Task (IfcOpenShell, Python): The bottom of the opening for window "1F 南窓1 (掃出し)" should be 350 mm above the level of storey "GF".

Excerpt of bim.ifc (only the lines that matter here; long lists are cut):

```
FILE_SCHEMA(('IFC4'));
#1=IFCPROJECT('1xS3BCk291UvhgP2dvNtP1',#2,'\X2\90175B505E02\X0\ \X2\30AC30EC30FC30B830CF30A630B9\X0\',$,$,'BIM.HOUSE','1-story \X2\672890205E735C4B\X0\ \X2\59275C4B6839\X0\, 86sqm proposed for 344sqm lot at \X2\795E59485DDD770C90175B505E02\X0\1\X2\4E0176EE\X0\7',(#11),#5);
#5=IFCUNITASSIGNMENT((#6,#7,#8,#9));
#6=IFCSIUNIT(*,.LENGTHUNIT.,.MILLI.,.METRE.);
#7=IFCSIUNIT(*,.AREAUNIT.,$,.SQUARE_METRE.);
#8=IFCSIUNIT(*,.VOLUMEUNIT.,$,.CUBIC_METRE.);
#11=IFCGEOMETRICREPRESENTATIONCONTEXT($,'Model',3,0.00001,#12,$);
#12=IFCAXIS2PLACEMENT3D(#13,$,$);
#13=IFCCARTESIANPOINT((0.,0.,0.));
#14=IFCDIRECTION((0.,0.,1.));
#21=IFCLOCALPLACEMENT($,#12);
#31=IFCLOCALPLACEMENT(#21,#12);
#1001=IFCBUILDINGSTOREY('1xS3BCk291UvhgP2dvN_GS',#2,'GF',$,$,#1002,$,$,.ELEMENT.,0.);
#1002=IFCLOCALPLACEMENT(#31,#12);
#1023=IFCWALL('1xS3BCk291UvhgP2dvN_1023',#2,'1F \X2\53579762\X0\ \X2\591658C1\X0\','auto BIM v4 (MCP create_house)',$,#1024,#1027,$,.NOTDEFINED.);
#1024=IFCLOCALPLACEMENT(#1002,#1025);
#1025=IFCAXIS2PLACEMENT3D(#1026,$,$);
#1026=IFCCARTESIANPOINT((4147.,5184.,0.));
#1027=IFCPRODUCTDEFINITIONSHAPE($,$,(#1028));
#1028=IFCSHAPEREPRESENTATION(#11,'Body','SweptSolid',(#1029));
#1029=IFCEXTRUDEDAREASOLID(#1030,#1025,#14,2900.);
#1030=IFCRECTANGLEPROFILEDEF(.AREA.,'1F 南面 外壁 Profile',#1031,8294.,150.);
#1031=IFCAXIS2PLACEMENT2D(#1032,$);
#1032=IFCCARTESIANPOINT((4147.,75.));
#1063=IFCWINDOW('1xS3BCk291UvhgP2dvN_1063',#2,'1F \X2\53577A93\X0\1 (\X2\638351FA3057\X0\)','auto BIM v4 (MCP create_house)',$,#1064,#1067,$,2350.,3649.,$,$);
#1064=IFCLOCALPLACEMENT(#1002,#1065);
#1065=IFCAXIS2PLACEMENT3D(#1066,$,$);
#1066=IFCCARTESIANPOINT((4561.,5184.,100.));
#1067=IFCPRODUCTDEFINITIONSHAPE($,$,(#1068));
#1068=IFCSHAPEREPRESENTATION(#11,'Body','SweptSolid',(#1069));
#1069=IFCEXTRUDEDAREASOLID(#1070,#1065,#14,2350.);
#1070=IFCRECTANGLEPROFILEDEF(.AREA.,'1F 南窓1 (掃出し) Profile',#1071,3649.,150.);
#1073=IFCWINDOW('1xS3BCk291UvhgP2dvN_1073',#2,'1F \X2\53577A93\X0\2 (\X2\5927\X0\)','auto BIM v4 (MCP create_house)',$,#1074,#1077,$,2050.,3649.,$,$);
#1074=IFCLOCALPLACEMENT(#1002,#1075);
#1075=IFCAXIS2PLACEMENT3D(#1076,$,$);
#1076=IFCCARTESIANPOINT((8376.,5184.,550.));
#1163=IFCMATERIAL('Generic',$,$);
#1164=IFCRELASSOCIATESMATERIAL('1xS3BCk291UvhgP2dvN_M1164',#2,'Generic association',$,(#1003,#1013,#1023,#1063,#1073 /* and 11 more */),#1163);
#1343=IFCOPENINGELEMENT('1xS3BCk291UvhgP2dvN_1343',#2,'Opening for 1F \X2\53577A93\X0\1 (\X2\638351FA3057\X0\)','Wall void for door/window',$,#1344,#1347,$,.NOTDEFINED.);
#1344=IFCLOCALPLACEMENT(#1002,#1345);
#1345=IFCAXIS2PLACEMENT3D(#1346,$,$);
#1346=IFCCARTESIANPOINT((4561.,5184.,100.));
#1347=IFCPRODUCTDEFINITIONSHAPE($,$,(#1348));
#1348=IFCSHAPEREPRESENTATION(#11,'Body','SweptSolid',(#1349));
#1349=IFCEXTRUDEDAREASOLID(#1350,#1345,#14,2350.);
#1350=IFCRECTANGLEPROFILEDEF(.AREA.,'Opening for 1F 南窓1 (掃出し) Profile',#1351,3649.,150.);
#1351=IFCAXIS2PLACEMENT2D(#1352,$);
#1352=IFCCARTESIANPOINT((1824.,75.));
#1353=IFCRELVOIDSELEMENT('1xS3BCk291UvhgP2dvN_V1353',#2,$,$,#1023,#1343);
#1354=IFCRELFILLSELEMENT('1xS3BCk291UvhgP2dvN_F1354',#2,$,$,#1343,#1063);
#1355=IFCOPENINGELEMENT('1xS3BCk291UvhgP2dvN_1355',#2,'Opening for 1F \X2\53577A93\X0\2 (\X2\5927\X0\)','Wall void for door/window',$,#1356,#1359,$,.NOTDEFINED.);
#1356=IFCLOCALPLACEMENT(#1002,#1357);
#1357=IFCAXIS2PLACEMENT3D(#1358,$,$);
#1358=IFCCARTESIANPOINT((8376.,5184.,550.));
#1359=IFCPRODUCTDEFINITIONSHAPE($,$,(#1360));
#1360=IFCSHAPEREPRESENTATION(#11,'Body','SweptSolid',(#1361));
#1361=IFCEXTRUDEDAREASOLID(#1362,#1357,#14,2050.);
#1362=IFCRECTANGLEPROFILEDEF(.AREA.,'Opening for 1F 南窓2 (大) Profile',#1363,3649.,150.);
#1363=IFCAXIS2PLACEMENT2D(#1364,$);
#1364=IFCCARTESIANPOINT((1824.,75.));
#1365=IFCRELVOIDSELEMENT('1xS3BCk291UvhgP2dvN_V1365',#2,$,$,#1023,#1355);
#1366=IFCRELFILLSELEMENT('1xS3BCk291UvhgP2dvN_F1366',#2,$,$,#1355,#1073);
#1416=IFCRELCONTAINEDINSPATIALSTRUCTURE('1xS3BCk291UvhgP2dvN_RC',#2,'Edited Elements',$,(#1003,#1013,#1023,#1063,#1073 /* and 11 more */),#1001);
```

```python
import numpy as np
import ifcopenshell
import ifcopenshell.api.geometry
import ifcopenshell.geom
import ifcopenshell.util.element
import ifcopenshell.util.placement
import ifcopenshell.util.shape
import ifcopenshell.util.unit

model = ifcopenshell.open("bim.ifc")
unit_scale = ifcopenshell.util.unit.calculate_unit_scale(model)

window = model.by_guid("1xS3BCk291UvhgP2dvN_1063")
opening = window.FillsVoids[0].RelatingOpeningElement
storey = ifcopenshell.util.element.get_container(window, ifc_class="IfcBuildingStorey")
level = ifcopenshell.util.placement.get_local_placement(storey.ObjectPlacement)[2, 3]

# The opening's origin need not be at the sill, so measure its lowest point.
shape = ifcopenshell.geom.create_shape(ifcopenshell.geom.settings(), opening)
bottom = ifcopenshell.util.shape.get_shape_bottom_elevation(shape, shape.geometry) / unit_scale
dz = level + 350.0 - bottom

shift = np.array([0.0, 0.0, dz])
# The window is not placed relative to its opening, so move both.
for product in (opening, window):
    matrix = ifcopenshell.util.placement.get_local_placement(product.ObjectPlacement)
    matrix[:3, 3] += shift
    ifcopenshell.api.geometry.edit_object_placement(model, product=product, matrix=matrix, is_si=False)

print(f"moved by {dz * unit_scale:+.3f} m")

model.write("bim_rev.ifc")
```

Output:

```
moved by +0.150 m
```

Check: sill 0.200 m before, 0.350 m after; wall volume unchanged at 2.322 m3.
